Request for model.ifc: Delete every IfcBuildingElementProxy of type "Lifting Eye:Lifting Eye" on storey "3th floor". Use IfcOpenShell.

First a look at what the model holds.

```python
import ifcopenshell
import ifcopenshell.util.element

model = ifcopenshell.open("model.ifc")
print(model.schema)
storey = next(s for s in model.by_type("IfcBuildingStorey") if s.Name == "3th floor")
proxies = [e for e in ifcopenshell.util.element.get_decomposition(storey) if e.is_a("IfcBuildingElementProxy")]
seen = {}
for e in proxies:
    element_type = ifcopenshell.util.element.get_type(e)
    name = element_type.Name if element_type not in (None, e) else None
    seen[name] = seen.get(name, 0) + 1
for name, count in sorted(seen.items(), key=str):
    print(count, "x", name)
```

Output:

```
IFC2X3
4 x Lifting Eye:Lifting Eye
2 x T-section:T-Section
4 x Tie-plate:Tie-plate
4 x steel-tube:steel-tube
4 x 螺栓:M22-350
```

```python
import ifcopenshell
import ifcopenshell.api.root
import ifcopenshell.util.element

model = ifcopenshell.open("model.ifc")

storey = next(s for s in model.by_type("IfcBuildingStorey") if s.Name == "3th floor")
proxies = [e for e in ifcopenshell.util.element.get_decomposition(storey) if e.is_a("IfcBuildingElementProxy")]
targets = [e for e in proxies if (t := ifcopenshell.util.element.get_type(e)) not in (None, e) and t.Name == "Lifting Eye:Lifting Eye"]

for e in targets:
    ifcopenshell.api.root.remove_product(model, product=e)
print(len(targets), "removed")

model.write("model_v2.ifc")
```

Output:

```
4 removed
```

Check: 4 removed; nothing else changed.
